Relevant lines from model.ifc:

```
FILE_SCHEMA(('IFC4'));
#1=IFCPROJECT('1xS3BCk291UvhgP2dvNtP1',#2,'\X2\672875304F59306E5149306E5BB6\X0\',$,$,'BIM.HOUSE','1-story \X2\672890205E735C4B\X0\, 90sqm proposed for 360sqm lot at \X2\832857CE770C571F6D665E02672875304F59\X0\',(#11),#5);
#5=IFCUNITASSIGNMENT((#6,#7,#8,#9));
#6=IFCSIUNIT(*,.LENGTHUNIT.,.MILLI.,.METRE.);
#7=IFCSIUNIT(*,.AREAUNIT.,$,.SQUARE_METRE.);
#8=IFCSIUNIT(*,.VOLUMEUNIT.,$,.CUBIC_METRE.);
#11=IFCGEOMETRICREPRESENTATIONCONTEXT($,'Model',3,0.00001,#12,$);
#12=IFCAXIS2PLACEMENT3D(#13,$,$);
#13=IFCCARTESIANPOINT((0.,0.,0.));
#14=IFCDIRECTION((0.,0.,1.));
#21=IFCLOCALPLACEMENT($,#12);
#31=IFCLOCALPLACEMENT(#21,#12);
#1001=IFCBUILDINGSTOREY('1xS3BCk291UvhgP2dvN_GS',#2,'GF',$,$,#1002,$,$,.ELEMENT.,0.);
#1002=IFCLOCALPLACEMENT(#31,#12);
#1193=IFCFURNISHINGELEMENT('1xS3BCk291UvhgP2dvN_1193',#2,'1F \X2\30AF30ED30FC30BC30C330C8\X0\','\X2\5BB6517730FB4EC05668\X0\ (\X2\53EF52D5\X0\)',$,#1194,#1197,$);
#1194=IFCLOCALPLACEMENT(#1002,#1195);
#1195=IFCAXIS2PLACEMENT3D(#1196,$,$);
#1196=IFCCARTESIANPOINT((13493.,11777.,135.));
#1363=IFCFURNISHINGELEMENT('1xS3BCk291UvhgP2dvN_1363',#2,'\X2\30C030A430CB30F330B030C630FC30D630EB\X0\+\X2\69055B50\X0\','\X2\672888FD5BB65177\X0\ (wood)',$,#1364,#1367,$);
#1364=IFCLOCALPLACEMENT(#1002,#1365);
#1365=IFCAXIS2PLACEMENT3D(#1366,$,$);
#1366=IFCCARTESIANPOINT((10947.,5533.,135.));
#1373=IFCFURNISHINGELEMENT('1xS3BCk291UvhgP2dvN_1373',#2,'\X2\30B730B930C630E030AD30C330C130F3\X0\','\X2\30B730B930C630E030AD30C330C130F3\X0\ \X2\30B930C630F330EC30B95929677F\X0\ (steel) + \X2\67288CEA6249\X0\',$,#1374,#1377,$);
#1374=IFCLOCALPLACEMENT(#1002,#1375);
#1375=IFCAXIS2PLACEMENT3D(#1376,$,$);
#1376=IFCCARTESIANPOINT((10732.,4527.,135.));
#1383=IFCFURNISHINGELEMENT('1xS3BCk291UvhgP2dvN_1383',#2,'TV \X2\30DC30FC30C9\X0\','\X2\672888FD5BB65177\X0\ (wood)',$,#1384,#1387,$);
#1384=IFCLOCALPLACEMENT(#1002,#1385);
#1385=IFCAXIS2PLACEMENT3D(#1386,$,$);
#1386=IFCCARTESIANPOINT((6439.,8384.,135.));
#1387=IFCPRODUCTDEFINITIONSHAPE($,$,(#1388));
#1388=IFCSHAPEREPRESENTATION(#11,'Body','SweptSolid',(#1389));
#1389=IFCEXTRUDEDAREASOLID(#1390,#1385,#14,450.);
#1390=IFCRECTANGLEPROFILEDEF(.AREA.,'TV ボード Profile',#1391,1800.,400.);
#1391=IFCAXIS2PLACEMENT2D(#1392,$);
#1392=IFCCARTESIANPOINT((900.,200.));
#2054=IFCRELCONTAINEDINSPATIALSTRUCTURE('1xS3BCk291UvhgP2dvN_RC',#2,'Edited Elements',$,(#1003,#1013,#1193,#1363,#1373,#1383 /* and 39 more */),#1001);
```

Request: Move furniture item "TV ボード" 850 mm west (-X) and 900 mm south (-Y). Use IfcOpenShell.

```python
import ifcopenshell
import ifcopenshell.api.geometry
import ifcopenshell.util.placement

model = ifcopenshell.open("model.ifc")

item = model.by_id(1383)
matrix = ifcopenshell.util.placement.get_local_placement(item.ObjectPlacement)
matrix[0, 3] -= 850.0
matrix[1, 3] -= 900.0
ifcopenshell.api.geometry.edit_object_placement(model, product=item, matrix=matrix, is_si=False)

print(ifcopenshell.util.placement.get_local_placement(item.ObjectPlacement).round(3) + 0.0)

model.write("model_v2.ifc")
```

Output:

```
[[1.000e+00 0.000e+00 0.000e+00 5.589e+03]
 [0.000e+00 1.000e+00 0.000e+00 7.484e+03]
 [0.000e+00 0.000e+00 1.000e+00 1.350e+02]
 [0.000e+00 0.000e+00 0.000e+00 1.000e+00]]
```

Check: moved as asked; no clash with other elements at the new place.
